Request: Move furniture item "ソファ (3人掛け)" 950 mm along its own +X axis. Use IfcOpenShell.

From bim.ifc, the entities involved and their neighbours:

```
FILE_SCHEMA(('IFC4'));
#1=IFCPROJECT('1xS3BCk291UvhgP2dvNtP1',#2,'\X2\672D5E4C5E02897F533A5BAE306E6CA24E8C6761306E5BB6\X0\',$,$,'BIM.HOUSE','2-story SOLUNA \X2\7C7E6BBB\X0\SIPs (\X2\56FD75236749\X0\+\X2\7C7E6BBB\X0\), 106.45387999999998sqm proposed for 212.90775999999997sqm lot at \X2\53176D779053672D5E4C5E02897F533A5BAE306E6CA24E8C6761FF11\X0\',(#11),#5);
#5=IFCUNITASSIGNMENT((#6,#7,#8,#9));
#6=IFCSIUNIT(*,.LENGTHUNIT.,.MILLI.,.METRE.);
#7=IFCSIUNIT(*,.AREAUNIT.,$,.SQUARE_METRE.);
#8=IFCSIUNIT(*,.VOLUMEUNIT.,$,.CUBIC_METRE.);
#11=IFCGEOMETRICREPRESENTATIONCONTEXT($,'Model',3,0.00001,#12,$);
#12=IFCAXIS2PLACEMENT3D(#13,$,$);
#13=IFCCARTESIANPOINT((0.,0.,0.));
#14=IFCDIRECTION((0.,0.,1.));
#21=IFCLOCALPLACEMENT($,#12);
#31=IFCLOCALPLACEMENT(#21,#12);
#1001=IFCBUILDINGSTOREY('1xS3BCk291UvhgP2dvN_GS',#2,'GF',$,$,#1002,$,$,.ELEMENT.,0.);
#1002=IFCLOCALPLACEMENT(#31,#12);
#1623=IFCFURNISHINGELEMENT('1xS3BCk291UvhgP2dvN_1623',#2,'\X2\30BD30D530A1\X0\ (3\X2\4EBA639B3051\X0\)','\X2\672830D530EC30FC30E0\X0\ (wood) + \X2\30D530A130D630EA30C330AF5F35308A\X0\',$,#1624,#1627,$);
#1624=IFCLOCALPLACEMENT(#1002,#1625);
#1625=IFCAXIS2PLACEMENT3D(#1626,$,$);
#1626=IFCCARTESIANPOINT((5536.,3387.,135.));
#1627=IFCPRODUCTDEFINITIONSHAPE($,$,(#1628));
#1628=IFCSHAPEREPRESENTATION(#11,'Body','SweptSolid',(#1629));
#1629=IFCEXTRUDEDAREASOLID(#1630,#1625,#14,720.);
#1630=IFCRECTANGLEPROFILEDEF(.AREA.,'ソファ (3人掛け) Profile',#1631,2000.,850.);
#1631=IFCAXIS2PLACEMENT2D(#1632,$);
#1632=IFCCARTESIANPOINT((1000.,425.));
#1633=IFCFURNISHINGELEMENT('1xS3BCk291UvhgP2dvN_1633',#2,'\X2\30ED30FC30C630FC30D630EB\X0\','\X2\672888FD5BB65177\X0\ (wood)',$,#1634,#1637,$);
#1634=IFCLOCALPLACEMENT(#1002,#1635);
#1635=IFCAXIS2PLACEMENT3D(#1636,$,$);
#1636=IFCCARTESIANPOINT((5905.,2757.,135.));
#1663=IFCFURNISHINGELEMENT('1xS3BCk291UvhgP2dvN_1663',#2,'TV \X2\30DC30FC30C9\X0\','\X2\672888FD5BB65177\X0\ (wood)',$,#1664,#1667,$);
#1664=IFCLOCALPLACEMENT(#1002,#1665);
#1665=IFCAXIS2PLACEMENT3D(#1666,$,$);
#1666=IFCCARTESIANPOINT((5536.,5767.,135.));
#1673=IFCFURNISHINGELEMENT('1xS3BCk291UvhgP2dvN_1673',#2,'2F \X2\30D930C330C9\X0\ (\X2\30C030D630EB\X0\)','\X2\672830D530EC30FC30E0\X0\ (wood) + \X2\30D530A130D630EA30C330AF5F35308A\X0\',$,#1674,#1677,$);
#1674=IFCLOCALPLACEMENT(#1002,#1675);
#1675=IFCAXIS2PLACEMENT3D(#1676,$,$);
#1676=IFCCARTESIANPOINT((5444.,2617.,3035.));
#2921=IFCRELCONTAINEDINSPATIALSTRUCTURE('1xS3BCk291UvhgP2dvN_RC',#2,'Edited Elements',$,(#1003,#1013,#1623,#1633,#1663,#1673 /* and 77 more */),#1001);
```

```python
import ifcopenshell
import ifcopenshell.api.geometry
import ifcopenshell.util.placement
import ifcopenshell.util.unit

model = ifcopenshell.open("bim.ifc")
unit_scale = ifcopenshell.util.unit.calculate_unit_scale(model)

item = model.by_guid("1xS3BCk291UvhgP2dvN_1623")
matrix = ifcopenshell.util.placement.get_local_placement(item.ObjectPlacement)
matrix[:3, 3] += matrix[:3, 0] * 0.95 / unit_scale
ifcopenshell.api.geometry.edit_object_placement(model, product=item, matrix=matrix, is_si=False)

print(ifcopenshell.util.placement.get_local_placement(item.ObjectPlacement).round(3) + 0.0)

model.write("bim_rev.ifc")
```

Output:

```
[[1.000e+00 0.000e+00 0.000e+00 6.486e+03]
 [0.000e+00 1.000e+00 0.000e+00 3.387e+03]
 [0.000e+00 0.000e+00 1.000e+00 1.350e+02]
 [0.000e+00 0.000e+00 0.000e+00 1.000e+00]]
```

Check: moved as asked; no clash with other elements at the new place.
